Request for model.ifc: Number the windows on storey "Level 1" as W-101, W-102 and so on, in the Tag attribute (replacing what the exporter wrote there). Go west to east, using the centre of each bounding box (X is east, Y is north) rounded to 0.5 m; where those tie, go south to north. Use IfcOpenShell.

First a look at what the model holds.

```python
import ifcopenshell
import ifcopenshell.util.element
import ifcopenshell.util.placement

model = ifcopenshell.open("model.ifc")
print(model.schema)
storey = next(s for s in model.by_type("IfcBuildingStorey") if s.Name == "Level 1")
windows = [e for e in ifcopenshell.util.element.get_decomposition(storey) if e.is_a("IfcWindow")]
for e in sorted(windows, key=lambda e: e.id()):
    origin = ifcopenshell.util.placement.get_local_placement(e.ObjectPlacement)[:3, 3]
    print(e.id(), e.Tag, e.Name, origin.round(2) + 0.0, sep=" | ")
```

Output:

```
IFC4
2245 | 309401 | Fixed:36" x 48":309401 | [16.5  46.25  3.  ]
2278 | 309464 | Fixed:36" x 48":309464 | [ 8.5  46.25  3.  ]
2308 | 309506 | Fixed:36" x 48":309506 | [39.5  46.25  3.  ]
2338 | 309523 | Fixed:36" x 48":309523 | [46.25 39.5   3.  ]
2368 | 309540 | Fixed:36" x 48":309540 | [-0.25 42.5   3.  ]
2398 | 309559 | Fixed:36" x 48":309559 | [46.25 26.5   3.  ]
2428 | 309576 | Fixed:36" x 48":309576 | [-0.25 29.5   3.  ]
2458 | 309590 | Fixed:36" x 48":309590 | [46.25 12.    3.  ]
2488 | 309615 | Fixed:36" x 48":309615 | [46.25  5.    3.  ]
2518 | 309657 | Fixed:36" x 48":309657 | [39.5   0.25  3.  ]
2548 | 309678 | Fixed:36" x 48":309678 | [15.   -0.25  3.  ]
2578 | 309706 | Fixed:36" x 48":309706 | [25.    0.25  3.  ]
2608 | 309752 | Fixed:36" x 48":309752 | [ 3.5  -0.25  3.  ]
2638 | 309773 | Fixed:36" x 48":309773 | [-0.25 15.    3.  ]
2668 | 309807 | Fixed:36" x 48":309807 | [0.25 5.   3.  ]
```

```python
import ifcopenshell
import ifcopenshell.geom
import ifcopenshell.util.element
import ifcopenshell.util.shape

model = ifcopenshell.open("model.ifc")
settings = ifcopenshell.geom.settings()
settings.set("use-world-coords", True)


def centre(element):
    shape = ifcopenshell.geom.create_shape(settings, element)
    return ifcopenshell.util.shape.get_bbox_centroid(shape.geometry)


storey = next(s for s in model.by_type("IfcBuildingStorey") if s.Name == "Level 1")
windows = [e for e in ifcopenshell.util.element.get_decomposition(storey) if e.is_a("IfcWindow")]

# Insertion points can sit at a corner or the storey origin, so sort by the geometry (in metres).
centres = {e: centre(e) for e in windows}
windows.sort(key=lambda e: (round(centres[e][0] / 0.5), centres[e][1]))

for i, e in enumerate(windows, start=1):
    number = f"W-1{i:02d}"
    e.Tag = number
    print(e.id(), number)

model.write("model_updated.ifc")
```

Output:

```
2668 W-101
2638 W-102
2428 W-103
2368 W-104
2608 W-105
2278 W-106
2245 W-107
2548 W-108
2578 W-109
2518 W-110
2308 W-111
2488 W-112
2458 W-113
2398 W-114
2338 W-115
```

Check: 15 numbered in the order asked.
